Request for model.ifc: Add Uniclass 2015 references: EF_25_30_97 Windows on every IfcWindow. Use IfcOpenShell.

First a look at what the model holds.

```python
import ifcopenshell

model = ifcopenshell.open("model.ifc")
print(model.schema)
print("classifications:", [c.Name for c in model.by_type("IfcClassification")])
for ifc_class in ("IfcDoor", "IfcRoof", "IfcStair", "IfcWall", "IfcWindow"):
    print(ifc_class, len(model.by_type(ifc_class)))
```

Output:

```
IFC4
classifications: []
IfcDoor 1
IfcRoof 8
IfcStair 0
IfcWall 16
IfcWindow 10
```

```python
import ifcopenshell
import ifcopenshell.api.classification

model = ifcopenshell.open("model.ifc")

system = ifcopenshell.api.classification.add_classification(model, classification="Uniclass 2015")

codes = {
    "IfcWindow": ("EF_25_30_97", "Windows"),
}
for ifc_class, (code, name) in codes.items():
    products = model.by_type(ifc_class)
    ifcopenshell.api.classification.add_reference(
        model, products=products, classification=system, identification=code, name=name
    )
    print(code, len(products))

model.write("model_v2.ifc")
```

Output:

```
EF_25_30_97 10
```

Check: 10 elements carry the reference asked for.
